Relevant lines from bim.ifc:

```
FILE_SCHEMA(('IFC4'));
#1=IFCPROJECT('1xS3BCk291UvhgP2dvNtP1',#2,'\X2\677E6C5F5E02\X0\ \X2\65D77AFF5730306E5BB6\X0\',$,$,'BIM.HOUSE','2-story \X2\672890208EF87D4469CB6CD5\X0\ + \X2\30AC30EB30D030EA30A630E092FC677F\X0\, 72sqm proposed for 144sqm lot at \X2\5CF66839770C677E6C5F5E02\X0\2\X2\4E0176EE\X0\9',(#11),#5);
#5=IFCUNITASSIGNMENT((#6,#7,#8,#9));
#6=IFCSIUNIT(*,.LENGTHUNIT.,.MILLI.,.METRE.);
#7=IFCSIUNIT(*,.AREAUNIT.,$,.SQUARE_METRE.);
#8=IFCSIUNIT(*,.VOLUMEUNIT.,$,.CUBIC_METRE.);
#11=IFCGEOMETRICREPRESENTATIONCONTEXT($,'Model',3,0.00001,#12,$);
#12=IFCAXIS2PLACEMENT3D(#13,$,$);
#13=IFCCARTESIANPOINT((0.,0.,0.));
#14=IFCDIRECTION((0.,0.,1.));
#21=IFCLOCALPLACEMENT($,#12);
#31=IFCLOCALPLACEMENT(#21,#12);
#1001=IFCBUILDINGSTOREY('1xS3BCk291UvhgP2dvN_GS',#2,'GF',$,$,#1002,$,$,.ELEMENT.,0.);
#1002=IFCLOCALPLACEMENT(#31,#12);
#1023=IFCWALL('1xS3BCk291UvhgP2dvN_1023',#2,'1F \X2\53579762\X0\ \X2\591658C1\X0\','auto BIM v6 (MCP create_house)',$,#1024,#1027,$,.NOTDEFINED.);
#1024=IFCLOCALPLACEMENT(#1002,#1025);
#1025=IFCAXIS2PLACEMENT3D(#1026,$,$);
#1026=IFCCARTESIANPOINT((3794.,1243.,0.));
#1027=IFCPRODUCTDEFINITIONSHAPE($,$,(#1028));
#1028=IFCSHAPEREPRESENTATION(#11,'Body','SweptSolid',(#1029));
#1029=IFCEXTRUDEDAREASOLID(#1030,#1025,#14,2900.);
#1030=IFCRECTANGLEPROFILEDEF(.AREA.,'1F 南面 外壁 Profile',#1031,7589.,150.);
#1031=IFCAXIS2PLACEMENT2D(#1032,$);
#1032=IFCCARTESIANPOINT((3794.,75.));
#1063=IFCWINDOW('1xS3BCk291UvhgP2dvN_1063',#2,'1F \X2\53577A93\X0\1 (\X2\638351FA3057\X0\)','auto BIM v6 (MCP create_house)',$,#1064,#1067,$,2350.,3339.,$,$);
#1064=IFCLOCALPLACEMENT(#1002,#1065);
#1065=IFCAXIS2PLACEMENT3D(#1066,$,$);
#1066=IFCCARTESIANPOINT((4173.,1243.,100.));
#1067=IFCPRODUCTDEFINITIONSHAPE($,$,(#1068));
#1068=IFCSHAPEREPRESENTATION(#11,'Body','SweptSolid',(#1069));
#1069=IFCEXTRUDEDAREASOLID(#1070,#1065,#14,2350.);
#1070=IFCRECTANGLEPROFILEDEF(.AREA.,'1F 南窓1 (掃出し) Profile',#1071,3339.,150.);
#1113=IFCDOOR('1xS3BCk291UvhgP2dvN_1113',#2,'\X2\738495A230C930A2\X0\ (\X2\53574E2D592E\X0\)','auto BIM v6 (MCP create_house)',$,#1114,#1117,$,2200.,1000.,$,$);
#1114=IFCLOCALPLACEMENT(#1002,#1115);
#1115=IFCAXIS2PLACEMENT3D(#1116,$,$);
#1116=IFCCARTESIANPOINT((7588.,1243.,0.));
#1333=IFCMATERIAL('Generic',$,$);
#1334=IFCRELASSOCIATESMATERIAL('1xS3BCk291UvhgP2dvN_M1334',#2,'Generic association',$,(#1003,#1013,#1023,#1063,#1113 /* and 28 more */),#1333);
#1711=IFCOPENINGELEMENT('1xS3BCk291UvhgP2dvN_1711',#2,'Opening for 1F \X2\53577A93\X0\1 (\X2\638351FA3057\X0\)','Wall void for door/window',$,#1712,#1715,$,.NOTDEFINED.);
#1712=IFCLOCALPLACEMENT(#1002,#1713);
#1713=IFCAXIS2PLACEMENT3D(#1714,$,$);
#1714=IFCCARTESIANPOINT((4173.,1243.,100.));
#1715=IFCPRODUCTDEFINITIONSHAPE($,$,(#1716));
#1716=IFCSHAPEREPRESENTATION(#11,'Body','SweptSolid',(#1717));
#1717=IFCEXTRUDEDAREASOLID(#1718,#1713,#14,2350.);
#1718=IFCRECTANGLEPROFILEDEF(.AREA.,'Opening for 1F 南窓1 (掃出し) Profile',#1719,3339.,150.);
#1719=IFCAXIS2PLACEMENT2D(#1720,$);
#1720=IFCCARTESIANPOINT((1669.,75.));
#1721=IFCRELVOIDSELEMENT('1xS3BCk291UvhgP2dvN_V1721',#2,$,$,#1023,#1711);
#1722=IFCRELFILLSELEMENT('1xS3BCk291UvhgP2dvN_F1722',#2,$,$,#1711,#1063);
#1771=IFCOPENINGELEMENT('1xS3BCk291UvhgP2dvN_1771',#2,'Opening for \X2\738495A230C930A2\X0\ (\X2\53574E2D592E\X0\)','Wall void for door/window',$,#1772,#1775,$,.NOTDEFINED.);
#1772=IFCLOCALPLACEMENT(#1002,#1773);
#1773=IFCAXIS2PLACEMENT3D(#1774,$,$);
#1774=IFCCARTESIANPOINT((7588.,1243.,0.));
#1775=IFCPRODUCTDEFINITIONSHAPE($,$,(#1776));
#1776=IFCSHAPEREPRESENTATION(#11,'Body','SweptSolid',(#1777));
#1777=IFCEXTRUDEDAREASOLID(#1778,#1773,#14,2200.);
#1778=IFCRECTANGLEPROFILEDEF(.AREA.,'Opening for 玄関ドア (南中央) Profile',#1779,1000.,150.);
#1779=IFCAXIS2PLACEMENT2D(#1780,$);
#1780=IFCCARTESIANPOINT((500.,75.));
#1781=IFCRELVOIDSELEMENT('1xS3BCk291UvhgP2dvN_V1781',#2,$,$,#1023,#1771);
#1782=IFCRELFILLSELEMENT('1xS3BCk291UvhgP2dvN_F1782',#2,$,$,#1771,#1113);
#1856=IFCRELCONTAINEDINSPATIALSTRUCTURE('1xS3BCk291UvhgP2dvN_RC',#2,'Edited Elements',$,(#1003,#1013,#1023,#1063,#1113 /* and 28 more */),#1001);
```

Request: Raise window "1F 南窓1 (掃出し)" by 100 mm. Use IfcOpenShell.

```python
import numpy as np
import ifcopenshell
import ifcopenshell.api.geometry
import ifcopenshell.util.placement
import ifcopenshell.util.unit

model = ifcopenshell.open("bim.ifc")
unit_scale = ifcopenshell.util.unit.calculate_unit_scale(model)

window = model.by_guid("1xS3BCk291UvhgP2dvN_1063")
opening = window.FillsVoids[0].RelatingOpeningElement
dz = 0.1 / unit_scale

shift = np.array([0.0, 0.0, dz])
# The window is not placed relative to its opening, so move both.
for product in (opening, window):
    matrix = ifcopenshell.util.placement.get_local_placement(product.ObjectPlacement)
    matrix[:3, 3] += shift
    ifcopenshell.api.geometry.edit_object_placement(model, product=product, matrix=matrix, is_si=False)

print(f"moved by {dz * unit_scale:+.3f} m")

model.write("bim-out.ifc")
```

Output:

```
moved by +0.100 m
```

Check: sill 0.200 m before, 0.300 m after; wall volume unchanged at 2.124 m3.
